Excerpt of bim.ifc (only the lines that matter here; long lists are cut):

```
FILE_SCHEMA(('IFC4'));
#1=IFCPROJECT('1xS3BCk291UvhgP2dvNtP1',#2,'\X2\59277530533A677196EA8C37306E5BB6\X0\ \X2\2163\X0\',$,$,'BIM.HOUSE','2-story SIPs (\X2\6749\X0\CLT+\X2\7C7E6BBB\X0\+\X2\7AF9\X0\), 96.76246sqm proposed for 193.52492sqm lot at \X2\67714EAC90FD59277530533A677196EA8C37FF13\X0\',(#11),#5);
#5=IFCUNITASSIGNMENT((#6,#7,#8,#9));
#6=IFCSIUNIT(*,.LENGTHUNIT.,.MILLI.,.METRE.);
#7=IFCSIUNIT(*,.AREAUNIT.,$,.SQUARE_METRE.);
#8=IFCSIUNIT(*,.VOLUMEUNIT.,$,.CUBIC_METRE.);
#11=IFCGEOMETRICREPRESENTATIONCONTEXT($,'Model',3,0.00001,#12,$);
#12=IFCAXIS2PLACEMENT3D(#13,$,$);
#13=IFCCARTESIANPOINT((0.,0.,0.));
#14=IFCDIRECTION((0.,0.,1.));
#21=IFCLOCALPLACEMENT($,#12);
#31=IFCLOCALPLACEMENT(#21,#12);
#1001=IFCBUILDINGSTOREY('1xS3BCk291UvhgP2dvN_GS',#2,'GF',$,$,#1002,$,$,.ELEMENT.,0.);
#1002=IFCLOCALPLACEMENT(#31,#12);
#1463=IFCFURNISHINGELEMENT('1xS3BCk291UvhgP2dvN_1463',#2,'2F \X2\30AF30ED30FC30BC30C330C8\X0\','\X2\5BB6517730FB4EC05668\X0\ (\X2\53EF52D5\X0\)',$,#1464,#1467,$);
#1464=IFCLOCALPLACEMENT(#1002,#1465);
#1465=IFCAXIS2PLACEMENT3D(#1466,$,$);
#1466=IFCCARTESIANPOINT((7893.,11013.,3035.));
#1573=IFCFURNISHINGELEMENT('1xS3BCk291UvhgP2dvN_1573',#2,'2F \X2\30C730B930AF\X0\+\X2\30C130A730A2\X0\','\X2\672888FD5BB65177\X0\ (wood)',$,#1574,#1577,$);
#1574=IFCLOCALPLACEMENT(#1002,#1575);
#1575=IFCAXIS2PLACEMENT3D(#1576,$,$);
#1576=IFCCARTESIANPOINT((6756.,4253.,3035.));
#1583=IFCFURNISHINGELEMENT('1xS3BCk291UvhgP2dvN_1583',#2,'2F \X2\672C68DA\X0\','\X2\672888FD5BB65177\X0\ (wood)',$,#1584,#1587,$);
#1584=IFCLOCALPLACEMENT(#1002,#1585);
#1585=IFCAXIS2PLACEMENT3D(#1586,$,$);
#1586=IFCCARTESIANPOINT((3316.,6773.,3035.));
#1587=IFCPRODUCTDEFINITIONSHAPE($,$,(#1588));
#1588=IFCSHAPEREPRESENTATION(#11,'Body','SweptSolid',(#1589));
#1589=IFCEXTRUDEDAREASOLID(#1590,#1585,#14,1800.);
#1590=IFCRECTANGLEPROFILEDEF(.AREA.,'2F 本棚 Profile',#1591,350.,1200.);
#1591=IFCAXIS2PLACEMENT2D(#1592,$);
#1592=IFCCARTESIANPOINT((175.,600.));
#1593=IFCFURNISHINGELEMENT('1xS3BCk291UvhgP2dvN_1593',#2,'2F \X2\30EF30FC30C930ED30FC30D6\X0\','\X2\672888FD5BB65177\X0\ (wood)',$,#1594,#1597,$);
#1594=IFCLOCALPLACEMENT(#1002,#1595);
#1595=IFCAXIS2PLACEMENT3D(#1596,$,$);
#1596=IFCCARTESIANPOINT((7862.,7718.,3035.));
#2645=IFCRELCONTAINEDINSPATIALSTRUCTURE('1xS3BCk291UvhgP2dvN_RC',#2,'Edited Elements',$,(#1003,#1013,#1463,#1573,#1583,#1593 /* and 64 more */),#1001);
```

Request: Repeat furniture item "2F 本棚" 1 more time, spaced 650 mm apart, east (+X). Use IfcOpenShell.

```python
import numpy as np
import ifcopenshell
import ifcopenshell.api.geometry
import ifcopenshell.api.root
import ifcopenshell.util.element
import ifcopenshell.util.placement
import ifcopenshell.util.unit

model = ifcopenshell.open("bim.ifc")
unit_scale = ifcopenshell.util.unit.calculate_unit_scale(model)


def reuse_history(source, copy):
    """copy_class also copies each property set's owner history, people and application; keep the originals."""
    for rel in copy.IsDefinedBy:
        if rel.is_a("IfcRelDefinesByProperties") and (history := rel.RelatingPropertyDefinition.OwnerHistory):
            rel.RelatingPropertyDefinition.OwnerHistory = source.OwnerHistory
            ifcopenshell.util.element.remove_deep2(model, history)


source = model.by_guid("1xS3BCk291UvhgP2dvN_1583")
base = ifcopenshell.util.placement.get_local_placement(source.ObjectPlacement)
step = np.array([1.0, 0.0, 0.0]) * 0.65 / unit_scale

for i in range(1, 2):
    copy = ifcopenshell.api.root.copy_class(model, product=source)
    copy.Representation = ifcopenshell.util.element.copy_deep(
        model, source.Representation, exclude=["IfcGeometricRepresentationContext", "IfcRepresentationMap"]
    )
    reuse_history(source, copy)
    matrix = base.copy()
    matrix[:3, 3] += i * step
    print("added at", matrix[:3, 3].round(3) + 0.0)
    ifcopenshell.api.geometry.edit_object_placement(model, product=copy, matrix=matrix, is_si=False)

model.write("bim_rev.ifc")
```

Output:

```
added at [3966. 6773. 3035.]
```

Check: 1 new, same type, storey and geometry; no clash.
